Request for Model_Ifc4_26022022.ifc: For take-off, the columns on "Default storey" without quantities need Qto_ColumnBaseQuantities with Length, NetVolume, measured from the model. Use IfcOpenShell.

First a look at what the model holds.

```python
import ifcopenshell
import ifcopenshell.util.element
import ifcopenshell.util.unit

model = ifcopenshell.open("Model_Ifc4_26022022.ifc")
print(model.schema)
for unit_type in ("LENGTHUNIT", "AREAUNIT", "VOLUMEUNIT"):
    print(unit_type, ifcopenshell.util.unit.calculate_unit_scale(model, unit_type))
storey = next(s for s in model.by_type("IfcBuildingStorey") if s.Name == "Default storey")
columns = [e for e in ifcopenshell.util.element.get_decomposition(storey) if e.is_a("IfcColumn")]
for e in sorted(columns, key=lambda e: e.id()):
    print(e.id(), e.is_a(), e.Name, list(ifcopenshell.util.element.get_psets(e, qtos_only=True)), sep=" | ")
```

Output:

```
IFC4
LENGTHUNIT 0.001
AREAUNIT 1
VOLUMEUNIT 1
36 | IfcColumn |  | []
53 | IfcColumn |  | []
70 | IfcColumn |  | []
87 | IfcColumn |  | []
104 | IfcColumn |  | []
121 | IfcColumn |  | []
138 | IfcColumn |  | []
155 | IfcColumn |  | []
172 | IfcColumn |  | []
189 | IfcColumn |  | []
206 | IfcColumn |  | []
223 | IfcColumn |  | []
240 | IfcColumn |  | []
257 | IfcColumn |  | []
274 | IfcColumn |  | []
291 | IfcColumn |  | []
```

```python
import ifcopenshell
import ifcopenshell.api.pset
import ifcopenshell.geom
import ifcopenshell.util.element
import ifcopenshell.util.shape
import ifcopenshell.util.unit

model = ifcopenshell.open("Model_Ifc4_26022022.ifc")
unit_scale = ifcopenshell.util.unit.calculate_unit_scale(model)
volume_scale = ifcopenshell.util.unit.calculate_unit_scale(model, "VOLUMEUNIT")
settings = ifcopenshell.geom.settings()

storey = next(s for s in model.by_type("IfcBuildingStorey") if s.Name == "Default storey")
columns = [e for e in ifcopenshell.util.element.get_decomposition(storey) if e.is_a("IfcColumn")]

for e in sorted(columns, key=lambda e: e.id()):
    if ifcopenshell.util.element.get_psets(e, qtos_only=True, should_inherit=False):
        continue
    # Geometry comes back in metres, in the element's own axes.
    shape = ifcopenshell.geom.create_shape(settings, e)
    values = {
        "Length": ifcopenshell.util.shape.get_z(shape.geometry) / unit_scale,
        "NetVolume": ifcopenshell.util.shape.get_volume(shape.geometry) / volume_scale,
    }
    qto = ifcopenshell.api.pset.add_qto(model, product=e, name="Qto_ColumnBaseQuantities")
    ifcopenshell.api.pset.edit_qto(model, qto=qto, properties=values)
    print(e.id(), {k: round(v, 3) for k, v in values.items()})

model.write("Model_Ifc4_26022022-out.ifc")
```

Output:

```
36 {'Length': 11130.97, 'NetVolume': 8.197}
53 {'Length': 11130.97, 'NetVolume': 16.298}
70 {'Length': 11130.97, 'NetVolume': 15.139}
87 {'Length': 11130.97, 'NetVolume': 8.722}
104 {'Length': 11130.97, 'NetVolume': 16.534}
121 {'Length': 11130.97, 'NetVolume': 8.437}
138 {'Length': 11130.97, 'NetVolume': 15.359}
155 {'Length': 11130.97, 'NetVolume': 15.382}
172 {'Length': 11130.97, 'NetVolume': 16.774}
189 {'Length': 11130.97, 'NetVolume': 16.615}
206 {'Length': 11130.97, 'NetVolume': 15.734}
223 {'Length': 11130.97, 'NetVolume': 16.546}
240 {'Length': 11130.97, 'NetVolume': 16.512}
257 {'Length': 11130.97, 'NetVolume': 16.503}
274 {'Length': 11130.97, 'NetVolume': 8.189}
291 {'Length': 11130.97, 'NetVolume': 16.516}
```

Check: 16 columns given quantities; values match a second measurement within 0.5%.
